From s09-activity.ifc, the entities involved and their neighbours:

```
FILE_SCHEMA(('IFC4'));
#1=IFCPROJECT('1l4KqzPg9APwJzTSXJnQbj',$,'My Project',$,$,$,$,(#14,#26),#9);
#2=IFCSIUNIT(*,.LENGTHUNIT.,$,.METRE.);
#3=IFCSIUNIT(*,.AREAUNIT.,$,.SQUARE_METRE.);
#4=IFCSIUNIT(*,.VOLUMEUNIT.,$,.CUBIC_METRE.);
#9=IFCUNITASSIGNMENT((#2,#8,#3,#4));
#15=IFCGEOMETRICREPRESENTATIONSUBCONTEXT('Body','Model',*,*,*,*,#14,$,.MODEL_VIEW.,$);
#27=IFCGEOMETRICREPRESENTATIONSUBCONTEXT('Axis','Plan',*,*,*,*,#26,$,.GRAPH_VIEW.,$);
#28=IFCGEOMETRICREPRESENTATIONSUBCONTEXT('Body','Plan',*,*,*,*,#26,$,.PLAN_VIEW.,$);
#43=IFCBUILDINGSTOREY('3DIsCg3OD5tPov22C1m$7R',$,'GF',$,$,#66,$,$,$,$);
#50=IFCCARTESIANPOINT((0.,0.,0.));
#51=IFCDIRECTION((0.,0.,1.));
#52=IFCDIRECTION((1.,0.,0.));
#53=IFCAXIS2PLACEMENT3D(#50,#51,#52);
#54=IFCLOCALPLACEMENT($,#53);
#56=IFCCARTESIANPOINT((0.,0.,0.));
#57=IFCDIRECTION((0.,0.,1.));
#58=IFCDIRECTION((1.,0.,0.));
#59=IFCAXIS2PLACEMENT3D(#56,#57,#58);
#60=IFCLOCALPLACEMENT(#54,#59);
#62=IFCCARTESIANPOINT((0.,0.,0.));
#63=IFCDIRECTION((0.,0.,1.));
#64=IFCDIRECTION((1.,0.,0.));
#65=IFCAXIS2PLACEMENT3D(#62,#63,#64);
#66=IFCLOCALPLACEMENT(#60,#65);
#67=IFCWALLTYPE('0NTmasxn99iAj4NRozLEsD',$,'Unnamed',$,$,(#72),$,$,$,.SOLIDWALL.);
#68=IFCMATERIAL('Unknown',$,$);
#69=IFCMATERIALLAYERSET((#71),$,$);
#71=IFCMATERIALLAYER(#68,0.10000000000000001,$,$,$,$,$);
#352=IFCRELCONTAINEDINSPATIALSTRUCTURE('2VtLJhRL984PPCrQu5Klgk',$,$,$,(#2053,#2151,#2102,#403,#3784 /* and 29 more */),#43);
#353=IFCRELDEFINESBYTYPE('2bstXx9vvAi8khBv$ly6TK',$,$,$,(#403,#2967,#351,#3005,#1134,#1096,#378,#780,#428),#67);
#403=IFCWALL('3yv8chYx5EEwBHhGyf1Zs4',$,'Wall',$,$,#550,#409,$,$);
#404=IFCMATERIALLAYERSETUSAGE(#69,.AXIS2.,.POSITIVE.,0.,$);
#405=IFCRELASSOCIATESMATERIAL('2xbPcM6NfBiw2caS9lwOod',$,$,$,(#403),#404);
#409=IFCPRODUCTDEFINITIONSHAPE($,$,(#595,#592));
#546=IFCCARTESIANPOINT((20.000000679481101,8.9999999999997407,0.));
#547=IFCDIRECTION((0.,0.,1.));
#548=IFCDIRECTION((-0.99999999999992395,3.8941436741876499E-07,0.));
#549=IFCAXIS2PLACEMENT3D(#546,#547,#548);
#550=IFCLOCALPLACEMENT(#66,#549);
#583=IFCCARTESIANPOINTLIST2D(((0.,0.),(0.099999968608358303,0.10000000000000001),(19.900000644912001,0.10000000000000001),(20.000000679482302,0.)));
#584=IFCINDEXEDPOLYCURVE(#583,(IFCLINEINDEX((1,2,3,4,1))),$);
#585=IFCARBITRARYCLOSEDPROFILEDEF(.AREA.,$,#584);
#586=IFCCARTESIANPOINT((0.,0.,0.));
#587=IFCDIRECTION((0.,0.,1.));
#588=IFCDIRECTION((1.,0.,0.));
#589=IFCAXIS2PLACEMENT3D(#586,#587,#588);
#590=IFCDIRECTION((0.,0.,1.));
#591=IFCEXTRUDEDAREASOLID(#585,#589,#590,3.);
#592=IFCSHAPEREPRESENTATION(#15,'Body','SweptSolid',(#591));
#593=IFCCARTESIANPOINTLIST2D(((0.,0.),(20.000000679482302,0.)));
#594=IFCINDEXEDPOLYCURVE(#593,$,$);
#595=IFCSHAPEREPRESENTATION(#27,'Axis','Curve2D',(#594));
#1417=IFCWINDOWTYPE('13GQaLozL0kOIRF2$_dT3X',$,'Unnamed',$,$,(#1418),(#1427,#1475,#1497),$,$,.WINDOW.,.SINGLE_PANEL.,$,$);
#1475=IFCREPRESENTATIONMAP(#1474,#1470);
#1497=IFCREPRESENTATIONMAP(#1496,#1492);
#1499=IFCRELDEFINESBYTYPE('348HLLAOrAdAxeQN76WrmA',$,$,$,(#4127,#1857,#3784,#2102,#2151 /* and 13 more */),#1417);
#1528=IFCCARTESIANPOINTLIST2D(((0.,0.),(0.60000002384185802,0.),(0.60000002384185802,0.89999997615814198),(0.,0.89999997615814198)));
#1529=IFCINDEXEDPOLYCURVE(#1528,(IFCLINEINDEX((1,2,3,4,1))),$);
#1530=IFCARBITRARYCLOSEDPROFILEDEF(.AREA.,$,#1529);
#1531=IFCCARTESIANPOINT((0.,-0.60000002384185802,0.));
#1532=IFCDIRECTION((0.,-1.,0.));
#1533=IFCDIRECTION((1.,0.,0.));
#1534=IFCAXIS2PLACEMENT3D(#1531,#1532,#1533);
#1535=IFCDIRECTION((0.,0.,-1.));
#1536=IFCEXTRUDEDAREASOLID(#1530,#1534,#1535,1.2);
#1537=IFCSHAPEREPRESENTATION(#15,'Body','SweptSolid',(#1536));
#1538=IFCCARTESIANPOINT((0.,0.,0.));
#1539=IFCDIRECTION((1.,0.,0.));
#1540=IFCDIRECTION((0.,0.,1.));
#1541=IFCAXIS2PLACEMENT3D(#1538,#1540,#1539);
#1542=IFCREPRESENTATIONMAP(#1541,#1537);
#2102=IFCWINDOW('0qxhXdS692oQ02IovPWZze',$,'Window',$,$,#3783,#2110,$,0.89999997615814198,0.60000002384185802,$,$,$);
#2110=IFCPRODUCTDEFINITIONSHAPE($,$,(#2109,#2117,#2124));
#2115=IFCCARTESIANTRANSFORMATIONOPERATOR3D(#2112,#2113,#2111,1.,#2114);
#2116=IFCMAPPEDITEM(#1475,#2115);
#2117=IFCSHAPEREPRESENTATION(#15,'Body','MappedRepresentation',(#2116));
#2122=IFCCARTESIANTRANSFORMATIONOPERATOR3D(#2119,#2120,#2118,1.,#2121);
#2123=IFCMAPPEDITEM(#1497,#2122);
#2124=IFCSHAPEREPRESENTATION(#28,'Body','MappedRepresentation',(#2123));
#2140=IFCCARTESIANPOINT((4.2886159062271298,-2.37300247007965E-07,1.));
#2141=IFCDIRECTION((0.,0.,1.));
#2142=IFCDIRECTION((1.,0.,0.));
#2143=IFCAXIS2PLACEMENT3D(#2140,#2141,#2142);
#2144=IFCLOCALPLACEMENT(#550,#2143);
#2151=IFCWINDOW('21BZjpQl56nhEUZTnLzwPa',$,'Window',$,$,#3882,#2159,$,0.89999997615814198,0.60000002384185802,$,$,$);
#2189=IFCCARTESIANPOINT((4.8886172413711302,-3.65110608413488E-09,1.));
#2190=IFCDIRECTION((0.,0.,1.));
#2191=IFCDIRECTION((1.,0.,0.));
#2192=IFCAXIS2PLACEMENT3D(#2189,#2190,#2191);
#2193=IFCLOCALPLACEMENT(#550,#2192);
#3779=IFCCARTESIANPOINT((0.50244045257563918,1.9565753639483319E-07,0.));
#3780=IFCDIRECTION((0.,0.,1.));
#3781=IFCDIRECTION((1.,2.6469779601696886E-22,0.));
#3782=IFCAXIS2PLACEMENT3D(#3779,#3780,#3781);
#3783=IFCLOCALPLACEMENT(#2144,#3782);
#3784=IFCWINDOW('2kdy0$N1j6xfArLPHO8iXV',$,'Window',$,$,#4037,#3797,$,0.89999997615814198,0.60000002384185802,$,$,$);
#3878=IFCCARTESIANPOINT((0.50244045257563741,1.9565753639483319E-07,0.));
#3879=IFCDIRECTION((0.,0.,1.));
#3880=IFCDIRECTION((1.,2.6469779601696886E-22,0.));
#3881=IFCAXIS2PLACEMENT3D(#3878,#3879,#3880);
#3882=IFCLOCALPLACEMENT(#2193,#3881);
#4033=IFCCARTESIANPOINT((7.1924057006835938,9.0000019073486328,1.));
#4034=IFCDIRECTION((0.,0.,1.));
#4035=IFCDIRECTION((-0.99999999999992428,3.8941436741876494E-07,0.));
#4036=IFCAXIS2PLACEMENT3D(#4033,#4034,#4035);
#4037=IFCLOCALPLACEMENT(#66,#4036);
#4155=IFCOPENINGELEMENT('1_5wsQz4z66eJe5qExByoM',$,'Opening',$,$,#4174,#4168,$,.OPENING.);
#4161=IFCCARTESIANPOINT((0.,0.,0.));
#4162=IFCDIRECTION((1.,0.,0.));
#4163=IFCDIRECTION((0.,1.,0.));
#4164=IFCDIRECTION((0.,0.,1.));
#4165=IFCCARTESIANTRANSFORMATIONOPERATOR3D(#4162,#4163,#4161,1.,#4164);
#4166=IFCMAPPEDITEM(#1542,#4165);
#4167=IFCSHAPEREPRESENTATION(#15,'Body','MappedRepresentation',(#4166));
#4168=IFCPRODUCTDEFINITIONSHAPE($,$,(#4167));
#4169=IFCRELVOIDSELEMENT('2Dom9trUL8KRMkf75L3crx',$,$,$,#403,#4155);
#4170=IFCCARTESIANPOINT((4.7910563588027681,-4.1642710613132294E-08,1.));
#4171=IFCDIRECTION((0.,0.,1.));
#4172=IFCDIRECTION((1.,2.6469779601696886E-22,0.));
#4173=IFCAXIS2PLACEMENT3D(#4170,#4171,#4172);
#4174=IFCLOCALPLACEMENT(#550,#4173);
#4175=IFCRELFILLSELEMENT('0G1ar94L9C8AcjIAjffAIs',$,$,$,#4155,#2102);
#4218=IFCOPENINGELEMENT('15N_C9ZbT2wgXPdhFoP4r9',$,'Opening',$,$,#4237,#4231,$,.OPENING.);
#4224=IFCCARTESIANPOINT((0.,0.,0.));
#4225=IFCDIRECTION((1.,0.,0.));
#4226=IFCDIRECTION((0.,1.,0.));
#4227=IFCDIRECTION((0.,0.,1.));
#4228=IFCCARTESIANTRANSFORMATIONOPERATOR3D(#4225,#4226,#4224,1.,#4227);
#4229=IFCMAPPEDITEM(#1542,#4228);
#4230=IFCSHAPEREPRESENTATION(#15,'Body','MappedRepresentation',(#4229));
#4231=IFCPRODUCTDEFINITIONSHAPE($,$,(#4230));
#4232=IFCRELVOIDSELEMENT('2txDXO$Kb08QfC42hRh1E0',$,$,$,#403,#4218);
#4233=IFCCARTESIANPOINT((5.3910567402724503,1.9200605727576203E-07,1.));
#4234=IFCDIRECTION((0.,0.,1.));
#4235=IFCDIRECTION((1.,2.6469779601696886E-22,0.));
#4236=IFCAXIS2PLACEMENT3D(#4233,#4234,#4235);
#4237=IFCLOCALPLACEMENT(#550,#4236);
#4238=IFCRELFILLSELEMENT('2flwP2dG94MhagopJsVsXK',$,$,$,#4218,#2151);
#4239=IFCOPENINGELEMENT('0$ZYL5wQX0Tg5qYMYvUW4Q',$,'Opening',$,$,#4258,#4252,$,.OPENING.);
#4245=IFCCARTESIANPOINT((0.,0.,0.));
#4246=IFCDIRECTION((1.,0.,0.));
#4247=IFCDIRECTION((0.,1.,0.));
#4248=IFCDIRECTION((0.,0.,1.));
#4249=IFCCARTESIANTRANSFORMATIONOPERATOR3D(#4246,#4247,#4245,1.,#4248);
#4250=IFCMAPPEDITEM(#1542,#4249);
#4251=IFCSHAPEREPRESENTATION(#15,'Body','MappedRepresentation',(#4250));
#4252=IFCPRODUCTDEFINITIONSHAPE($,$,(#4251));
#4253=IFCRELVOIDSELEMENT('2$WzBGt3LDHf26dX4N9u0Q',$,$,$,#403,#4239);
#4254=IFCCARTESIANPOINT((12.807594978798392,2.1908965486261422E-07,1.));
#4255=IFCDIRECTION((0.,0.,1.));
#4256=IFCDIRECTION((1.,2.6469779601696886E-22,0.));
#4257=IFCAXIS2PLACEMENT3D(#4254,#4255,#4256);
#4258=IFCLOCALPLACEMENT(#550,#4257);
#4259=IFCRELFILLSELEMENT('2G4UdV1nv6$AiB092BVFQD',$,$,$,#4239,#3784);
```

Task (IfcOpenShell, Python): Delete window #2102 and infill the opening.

```python
import ifcopenshell
import ifcopenshell.api.feature
import ifcopenshell.api.root
import ifcopenshell.geom
import ifcopenshell.util.shape

model = ifcopenshell.open("s09-activity.ifc")
settings = ifcopenshell.geom.settings()


def volume(element):
    """Net volume in cubic metres, openings subtracted."""
    shape = ifcopenshell.geom.create_shape(settings, element)
    return ifcopenshell.util.shape.get_volume(shape.geometry)


window = model.by_guid("0qxhXdS692oQ02IovPWZze")
opening = window.FillsVoids[0].RelatingOpeningElement
wall = opening.VoidsElements[0].RelatingBuildingElement
before = volume(wall)

ifcopenshell.api.root.remove_product(model, product=window)
ifcopenshell.api.feature.remove_feature(model, feature=opening)

after = volume(wall)

print(f"wall volume {before:.3f} -> {after:.3f} m3")

model.write("s09-activity_updated.ifc")
```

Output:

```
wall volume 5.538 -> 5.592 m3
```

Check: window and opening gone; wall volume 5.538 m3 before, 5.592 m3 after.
